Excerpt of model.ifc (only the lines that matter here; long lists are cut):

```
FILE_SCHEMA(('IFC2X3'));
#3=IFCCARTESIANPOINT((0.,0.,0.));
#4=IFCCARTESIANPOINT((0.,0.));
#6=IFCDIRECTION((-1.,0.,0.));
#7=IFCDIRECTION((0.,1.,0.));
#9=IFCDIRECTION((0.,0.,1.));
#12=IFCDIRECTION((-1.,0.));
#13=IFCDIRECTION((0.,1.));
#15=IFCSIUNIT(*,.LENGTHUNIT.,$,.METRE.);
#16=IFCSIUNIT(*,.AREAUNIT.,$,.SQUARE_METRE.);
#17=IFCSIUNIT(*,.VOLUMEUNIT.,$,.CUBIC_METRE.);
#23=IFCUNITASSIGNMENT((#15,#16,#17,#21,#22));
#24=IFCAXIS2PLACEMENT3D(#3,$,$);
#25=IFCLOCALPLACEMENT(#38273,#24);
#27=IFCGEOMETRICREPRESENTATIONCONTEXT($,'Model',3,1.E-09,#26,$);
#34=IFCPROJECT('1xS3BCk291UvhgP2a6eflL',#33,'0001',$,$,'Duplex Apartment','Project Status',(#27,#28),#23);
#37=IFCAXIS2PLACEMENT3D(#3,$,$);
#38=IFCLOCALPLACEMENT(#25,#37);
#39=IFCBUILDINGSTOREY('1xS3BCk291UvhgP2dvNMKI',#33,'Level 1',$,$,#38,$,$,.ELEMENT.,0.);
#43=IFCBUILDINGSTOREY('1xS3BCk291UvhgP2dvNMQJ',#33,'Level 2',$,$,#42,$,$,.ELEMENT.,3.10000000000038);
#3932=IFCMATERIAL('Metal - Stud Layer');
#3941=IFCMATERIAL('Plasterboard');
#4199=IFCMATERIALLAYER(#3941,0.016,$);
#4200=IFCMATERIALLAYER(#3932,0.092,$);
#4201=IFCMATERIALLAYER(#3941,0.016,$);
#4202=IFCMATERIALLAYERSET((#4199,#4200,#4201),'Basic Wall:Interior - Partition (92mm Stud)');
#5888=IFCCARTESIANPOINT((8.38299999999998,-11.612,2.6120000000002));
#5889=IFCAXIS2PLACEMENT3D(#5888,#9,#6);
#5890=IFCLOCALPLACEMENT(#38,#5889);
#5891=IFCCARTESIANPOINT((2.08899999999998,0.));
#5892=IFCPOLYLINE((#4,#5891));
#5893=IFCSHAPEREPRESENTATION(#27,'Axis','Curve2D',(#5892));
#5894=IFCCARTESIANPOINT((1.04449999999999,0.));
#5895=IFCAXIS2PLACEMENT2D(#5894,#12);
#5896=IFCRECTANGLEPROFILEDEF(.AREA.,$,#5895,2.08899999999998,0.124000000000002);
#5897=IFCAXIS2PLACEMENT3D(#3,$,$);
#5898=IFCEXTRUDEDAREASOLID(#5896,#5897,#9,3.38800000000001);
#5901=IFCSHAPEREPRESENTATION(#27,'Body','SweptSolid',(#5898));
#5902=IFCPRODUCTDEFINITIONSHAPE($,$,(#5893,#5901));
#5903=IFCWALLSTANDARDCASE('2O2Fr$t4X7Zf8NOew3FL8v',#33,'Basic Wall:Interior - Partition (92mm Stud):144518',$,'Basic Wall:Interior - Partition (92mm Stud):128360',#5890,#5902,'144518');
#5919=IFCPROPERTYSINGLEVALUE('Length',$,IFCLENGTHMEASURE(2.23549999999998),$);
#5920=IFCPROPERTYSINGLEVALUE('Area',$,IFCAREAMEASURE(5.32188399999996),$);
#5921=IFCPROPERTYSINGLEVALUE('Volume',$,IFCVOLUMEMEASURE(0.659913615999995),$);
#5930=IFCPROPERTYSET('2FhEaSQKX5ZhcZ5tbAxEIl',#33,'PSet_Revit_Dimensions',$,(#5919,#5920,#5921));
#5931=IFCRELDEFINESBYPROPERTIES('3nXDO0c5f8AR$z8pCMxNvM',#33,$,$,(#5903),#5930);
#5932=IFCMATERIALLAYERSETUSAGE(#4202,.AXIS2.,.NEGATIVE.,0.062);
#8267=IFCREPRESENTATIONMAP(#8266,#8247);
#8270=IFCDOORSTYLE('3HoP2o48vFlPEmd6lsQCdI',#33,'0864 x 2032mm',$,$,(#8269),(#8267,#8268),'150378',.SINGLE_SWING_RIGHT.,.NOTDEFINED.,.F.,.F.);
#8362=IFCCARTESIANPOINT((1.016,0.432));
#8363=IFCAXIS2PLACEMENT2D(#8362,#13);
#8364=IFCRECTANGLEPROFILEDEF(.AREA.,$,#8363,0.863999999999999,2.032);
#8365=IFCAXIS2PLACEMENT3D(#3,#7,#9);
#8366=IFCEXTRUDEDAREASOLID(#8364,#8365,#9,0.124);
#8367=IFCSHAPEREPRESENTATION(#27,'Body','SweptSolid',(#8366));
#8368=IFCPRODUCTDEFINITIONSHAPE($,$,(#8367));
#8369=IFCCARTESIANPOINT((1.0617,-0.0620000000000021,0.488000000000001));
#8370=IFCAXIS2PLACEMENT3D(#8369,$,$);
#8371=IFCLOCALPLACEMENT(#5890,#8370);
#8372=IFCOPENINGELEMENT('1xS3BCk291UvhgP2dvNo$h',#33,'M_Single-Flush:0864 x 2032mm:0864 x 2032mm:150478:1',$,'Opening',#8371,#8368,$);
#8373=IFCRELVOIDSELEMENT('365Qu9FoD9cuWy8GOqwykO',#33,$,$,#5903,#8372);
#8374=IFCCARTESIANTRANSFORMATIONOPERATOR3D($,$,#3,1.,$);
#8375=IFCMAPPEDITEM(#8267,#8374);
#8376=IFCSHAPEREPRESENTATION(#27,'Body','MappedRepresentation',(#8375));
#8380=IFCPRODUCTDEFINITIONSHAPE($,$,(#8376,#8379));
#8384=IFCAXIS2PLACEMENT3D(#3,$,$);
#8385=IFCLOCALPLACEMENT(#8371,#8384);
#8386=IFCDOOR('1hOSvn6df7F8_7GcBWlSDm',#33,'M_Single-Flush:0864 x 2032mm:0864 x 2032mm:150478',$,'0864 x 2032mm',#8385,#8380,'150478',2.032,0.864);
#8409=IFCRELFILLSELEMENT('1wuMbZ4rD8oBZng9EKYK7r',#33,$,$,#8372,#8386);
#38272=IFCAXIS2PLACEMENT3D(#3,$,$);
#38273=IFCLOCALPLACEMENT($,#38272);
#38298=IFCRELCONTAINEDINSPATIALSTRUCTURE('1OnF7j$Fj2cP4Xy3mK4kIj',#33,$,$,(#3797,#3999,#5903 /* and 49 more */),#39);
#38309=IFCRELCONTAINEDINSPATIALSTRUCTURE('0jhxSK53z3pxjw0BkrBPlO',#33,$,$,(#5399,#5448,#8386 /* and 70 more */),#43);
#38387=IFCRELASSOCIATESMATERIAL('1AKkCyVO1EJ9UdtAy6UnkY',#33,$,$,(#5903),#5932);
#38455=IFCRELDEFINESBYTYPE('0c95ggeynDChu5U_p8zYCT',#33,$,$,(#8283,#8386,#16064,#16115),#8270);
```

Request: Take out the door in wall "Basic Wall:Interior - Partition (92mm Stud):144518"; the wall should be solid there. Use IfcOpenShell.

```python
import ifcopenshell
import ifcopenshell.api.feature
import ifcopenshell.api.pset
import ifcopenshell.api.root
import ifcopenshell.geom
import ifcopenshell.util.element
import ifcopenshell.util.shape
import ifcopenshell.util.unit

model = ifcopenshell.open("model.ifc")
area_scale = ifcopenshell.util.unit.calculate_unit_scale(model, "AREAUNIT")
volume_scale = ifcopenshell.util.unit.calculate_unit_scale(model, "VOLUMEUNIT")
settings = ifcopenshell.geom.settings()


def volume(element):
    """Net volume in cubic metres, openings subtracted."""
    shape = ifcopenshell.geom.create_shape(settings, element)
    return ifcopenshell.util.shape.get_volume(shape.geometry)


door = model.by_guid("1hOSvn6df7F8_7GcBWlSDm")
opening = door.FillsVoids[0].RelatingOpeningElement
wall = opening.VoidsElements[0].RelatingBuildingElement
before = volume(wall)

ifcopenshell.api.root.remove_product(model, product=door)
ifcopenshell.api.feature.remove_feature(model, feature=opening)

after = volume(wall)
thickness = 0.124  # wall thickness in metres

# Update the wall's stored quantities.
pset = model.by_id(ifcopenshell.util.element.get_pset(wall, "PSet_Revit_Dimensions", should_inherit=False)["id"])
ifcopenshell.api.pset.edit_pset(model, pset=pset, properties={
    "Area": model.create_entity("IfcAreaMeasure", after / thickness / area_scale),
    "Volume": model.create_entity("IfcVolumeMeasure", after / volume_scale),
})

print(f"wall volume {before:.3f} -> {after:.3f} m3")

model.write("model_v2.ifc")
```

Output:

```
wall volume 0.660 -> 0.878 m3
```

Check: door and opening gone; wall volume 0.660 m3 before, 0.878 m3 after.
